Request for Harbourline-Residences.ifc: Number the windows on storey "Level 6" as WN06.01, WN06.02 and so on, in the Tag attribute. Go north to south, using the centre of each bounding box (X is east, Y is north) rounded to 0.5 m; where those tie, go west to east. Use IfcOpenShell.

First a look at what the model holds.

```python
import ifcopenshell
import ifcopenshell.util.element
import ifcopenshell.util.placement

model = ifcopenshell.open("Harbourline-Residences.ifc")
print(model.schema)
storey = next(s for s in model.by_type("IfcBuildingStorey") if s.Name == "Level 6")
windows = [e for e in ifcopenshell.util.element.get_decomposition(storey) if e.is_a("IfcWindow")]
for e in sorted(windows, key=lambda e: e.id()):
    origin = ifcopenshell.util.placement.get_local_placement(e.ObjectPlacement)[:3, 3]
    print(e.id(), e.Tag, e.Name, origin.round(2) + 0.0, sep=" | ")
```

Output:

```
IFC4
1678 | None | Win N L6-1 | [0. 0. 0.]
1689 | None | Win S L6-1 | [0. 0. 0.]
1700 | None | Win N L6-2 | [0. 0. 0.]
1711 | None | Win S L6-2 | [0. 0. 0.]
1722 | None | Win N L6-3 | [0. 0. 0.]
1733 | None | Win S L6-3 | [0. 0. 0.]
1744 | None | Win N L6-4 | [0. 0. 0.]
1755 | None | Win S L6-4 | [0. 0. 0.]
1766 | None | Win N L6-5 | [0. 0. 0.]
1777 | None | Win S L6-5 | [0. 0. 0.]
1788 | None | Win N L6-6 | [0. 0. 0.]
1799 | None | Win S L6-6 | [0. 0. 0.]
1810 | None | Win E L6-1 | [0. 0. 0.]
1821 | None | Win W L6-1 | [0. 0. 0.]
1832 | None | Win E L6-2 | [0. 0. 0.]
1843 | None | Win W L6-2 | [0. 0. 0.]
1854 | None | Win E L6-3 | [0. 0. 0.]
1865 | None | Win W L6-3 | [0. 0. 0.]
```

```python
import ifcopenshell
import ifcopenshell.geom
import ifcopenshell.util.element
import ifcopenshell.util.shape

model = ifcopenshell.open("Harbourline-Residences.ifc")
settings = ifcopenshell.geom.settings()
settings.set("use-world-coords", True)


def centre(element):
    shape = ifcopenshell.geom.create_shape(settings, element)
    return ifcopenshell.util.shape.get_bbox_centroid(shape.geometry)


storey = next(s for s in model.by_type("IfcBuildingStorey") if s.Name == "Level 6")
windows = [e for e in ifcopenshell.util.element.get_decomposition(storey) if e.is_a("IfcWindow")]

# Insertion points can sit at a corner or the storey origin, so sort by the geometry (in metres).
centres = {e: centre(e) for e in windows}
windows.sort(key=lambda e: (-round(centres[e][1] / 0.5), centres[e][0]))

for i, e in enumerate(windows, start=1):
    number = f"WN06.{i:02d}"
    e.Tag = number
    print(e.id(), number)

model.write("Harbourline-Residences_v2.ifc")
```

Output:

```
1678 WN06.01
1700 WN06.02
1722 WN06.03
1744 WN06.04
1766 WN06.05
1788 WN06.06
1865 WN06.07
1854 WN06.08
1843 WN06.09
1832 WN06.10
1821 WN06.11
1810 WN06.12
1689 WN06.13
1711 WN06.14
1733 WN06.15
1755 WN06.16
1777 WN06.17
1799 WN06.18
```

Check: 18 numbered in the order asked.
